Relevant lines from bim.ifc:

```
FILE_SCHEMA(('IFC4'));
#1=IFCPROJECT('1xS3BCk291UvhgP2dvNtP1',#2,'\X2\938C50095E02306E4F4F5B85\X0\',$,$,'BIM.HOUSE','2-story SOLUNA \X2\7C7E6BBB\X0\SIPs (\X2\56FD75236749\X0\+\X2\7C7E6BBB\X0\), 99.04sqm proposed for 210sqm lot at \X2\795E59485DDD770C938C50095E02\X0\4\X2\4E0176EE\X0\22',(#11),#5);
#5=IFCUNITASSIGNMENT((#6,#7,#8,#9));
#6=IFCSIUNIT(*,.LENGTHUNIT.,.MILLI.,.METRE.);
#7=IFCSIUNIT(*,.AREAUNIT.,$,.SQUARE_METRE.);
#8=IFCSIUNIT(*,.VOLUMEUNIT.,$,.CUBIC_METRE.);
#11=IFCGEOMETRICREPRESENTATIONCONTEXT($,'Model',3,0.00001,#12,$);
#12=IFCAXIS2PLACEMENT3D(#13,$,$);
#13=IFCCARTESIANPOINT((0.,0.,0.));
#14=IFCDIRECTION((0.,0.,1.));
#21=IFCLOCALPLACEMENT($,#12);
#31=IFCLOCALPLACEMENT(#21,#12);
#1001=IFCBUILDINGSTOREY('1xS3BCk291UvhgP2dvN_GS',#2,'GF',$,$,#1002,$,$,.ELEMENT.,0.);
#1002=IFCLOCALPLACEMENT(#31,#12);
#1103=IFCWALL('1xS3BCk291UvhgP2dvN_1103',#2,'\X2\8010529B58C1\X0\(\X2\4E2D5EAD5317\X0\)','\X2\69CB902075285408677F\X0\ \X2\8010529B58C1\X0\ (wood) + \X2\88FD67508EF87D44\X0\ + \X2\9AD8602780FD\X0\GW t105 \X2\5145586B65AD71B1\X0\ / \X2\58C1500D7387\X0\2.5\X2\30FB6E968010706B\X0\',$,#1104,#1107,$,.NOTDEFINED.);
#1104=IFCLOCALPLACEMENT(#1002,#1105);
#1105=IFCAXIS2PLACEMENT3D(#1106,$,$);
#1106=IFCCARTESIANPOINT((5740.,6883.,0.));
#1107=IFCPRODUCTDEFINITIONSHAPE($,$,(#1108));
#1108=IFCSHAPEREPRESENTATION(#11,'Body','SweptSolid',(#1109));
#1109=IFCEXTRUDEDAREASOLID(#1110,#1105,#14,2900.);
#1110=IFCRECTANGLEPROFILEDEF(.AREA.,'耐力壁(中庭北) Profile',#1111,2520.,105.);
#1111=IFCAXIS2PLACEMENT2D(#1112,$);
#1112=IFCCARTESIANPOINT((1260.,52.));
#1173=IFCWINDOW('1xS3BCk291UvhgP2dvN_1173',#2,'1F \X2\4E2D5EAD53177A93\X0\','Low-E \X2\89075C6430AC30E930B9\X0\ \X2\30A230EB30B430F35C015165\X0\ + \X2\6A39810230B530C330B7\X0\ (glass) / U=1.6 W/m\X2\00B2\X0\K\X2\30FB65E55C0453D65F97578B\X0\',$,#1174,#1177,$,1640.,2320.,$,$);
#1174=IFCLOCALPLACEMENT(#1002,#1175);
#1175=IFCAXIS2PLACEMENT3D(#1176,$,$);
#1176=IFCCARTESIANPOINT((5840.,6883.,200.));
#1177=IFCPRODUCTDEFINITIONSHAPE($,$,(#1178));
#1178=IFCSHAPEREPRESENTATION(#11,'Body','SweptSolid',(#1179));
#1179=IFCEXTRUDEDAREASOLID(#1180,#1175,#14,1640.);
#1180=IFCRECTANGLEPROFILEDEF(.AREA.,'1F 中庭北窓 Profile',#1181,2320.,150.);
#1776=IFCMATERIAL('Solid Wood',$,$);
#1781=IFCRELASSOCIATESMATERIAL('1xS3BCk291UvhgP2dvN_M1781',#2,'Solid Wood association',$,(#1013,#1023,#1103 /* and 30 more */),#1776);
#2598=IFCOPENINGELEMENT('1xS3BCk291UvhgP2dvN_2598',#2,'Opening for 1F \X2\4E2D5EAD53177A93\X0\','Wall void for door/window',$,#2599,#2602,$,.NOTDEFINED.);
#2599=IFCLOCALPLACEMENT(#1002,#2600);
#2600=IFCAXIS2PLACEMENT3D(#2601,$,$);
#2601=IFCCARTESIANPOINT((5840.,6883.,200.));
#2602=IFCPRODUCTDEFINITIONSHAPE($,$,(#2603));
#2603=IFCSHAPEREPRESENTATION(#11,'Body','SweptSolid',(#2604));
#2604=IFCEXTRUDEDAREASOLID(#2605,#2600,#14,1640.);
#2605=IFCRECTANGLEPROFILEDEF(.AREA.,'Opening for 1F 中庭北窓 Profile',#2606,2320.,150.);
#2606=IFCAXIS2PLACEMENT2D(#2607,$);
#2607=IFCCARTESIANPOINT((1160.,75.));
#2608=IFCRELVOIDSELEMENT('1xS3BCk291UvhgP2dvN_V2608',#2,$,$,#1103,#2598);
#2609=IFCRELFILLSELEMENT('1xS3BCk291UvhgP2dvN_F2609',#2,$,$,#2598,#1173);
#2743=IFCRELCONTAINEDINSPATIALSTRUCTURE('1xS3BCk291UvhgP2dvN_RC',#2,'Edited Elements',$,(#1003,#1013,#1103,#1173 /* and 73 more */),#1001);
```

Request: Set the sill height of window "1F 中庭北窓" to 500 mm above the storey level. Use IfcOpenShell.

```python
import numpy as np
import ifcopenshell
import ifcopenshell.api.geometry
import ifcopenshell.geom
import ifcopenshell.util.element
import ifcopenshell.util.placement
import ifcopenshell.util.shape
import ifcopenshell.util.unit

model = ifcopenshell.open("bim.ifc")
unit_scale = ifcopenshell.util.unit.calculate_unit_scale(model)

window = model.by_id(1173)
opening = window.FillsVoids[0].RelatingOpeningElement
storey = ifcopenshell.util.element.get_container(window, ifc_class="IfcBuildingStorey")
level = ifcopenshell.util.placement.get_local_placement(storey.ObjectPlacement)[2, 3]

# The opening's origin need not be at the sill, so measure its lowest point.
shape = ifcopenshell.geom.create_shape(ifcopenshell.geom.settings(), opening)
bottom = ifcopenshell.util.shape.get_shape_bottom_elevation(shape, shape.geometry) / unit_scale
dz = level + 0.5 / unit_scale - bottom

shift = np.array([0.0, 0.0, dz])
# The window is not placed relative to its opening, so move both.
for product in (opening, window):
    matrix = ifcopenshell.util.placement.get_local_placement(product.ObjectPlacement)
    matrix[:3, 3] += shift
    ifcopenshell.api.geometry.edit_object_placement(model, product=product, matrix=matrix, is_si=False)

print(f"moved by {dz * unit_scale:+.3f} m")

model.write("bim_updated.ifc")
```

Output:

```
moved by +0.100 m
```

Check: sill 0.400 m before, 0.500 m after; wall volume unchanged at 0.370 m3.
